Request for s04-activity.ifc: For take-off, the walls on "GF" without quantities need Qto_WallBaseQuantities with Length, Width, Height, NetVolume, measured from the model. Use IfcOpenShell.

First a look at what the model holds.

```python
import ifcopenshell
import ifcopenshell.util.element
import ifcopenshell.util.unit

model = ifcopenshell.open("s04-activity.ifc")
print(model.schema)
for unit_type in ("LENGTHUNIT", "AREAUNIT", "VOLUMEUNIT"):
    print(unit_type, ifcopenshell.util.unit.calculate_unit_scale(model, unit_type))
storey = next(s for s in model.by_type("IfcBuildingStorey") if s.Name == "GF")
walls = [e for e in ifcopenshell.util.element.get_decomposition(storey) if e.is_a("IfcWall")]
for e in sorted(walls, key=lambda e: e.id()):
    print(e.id(), e.is_a(), e.Name, list(ifcopenshell.util.element.get_psets(e, qtos_only=True)), sep=" | ")
```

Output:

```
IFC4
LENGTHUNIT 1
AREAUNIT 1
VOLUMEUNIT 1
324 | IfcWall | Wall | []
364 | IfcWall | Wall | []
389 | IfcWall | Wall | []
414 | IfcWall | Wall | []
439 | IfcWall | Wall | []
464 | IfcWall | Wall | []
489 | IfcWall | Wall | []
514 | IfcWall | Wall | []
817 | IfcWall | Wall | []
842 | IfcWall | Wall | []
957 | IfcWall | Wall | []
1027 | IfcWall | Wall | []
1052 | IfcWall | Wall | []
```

```python
import ifcopenshell
import ifcopenshell.api.pset
import ifcopenshell.geom
import ifcopenshell.util.element
import ifcopenshell.util.shape
import ifcopenshell.util.unit

model = ifcopenshell.open("s04-activity.ifc")
unit_scale = ifcopenshell.util.unit.calculate_unit_scale(model)
volume_scale = ifcopenshell.util.unit.calculate_unit_scale(model, "VOLUMEUNIT")
settings = ifcopenshell.geom.settings()

storey = next(s for s in model.by_type("IfcBuildingStorey") if s.Name == "GF")
walls = [e for e in ifcopenshell.util.element.get_decomposition(storey) if e.is_a("IfcWall")]

for e in sorted(walls, key=lambda e: e.id()):
    if ifcopenshell.util.element.get_psets(e, qtos_only=True, should_inherit=False):
        continue
    # Geometry comes back in metres, in the element's own axes.
    shape = ifcopenshell.geom.create_shape(settings, e)
    values = {
        "Length": ifcopenshell.util.shape.get_x(shape.geometry) / unit_scale,
        "Width": ifcopenshell.util.shape.get_y(shape.geometry) / unit_scale,
        "Height": ifcopenshell.util.shape.get_z(shape.geometry) / unit_scale,
        "NetVolume": ifcopenshell.util.shape.get_volume(shape.geometry) / volume_scale,
    }
    qto = ifcopenshell.api.pset.add_qto(model, product=e, name="Qto_WallBaseQuantities")
    ifcopenshell.api.pset.edit_qto(model, qto=qto, properties=values)
    print(e.id(), {k: round(v, 3) for k, v in values.items()})

model.write("s04-activity_rev.ifc")
```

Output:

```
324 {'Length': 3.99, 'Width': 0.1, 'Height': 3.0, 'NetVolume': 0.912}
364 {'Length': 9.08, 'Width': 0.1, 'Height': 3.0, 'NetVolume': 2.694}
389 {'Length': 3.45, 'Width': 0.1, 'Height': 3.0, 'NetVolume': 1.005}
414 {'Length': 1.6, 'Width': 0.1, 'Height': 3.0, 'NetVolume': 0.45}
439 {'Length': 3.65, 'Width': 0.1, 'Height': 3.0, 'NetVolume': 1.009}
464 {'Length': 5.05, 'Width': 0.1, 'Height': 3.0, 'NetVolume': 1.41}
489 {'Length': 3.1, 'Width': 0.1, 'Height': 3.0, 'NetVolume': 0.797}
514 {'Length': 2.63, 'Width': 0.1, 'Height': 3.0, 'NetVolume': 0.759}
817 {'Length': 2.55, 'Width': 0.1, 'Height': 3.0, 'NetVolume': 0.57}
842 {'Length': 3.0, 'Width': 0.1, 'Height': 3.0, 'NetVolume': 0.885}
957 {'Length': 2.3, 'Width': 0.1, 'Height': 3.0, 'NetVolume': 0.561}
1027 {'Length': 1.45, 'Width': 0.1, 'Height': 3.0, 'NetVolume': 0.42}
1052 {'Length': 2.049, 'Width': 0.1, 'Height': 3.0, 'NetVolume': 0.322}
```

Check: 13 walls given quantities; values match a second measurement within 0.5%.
